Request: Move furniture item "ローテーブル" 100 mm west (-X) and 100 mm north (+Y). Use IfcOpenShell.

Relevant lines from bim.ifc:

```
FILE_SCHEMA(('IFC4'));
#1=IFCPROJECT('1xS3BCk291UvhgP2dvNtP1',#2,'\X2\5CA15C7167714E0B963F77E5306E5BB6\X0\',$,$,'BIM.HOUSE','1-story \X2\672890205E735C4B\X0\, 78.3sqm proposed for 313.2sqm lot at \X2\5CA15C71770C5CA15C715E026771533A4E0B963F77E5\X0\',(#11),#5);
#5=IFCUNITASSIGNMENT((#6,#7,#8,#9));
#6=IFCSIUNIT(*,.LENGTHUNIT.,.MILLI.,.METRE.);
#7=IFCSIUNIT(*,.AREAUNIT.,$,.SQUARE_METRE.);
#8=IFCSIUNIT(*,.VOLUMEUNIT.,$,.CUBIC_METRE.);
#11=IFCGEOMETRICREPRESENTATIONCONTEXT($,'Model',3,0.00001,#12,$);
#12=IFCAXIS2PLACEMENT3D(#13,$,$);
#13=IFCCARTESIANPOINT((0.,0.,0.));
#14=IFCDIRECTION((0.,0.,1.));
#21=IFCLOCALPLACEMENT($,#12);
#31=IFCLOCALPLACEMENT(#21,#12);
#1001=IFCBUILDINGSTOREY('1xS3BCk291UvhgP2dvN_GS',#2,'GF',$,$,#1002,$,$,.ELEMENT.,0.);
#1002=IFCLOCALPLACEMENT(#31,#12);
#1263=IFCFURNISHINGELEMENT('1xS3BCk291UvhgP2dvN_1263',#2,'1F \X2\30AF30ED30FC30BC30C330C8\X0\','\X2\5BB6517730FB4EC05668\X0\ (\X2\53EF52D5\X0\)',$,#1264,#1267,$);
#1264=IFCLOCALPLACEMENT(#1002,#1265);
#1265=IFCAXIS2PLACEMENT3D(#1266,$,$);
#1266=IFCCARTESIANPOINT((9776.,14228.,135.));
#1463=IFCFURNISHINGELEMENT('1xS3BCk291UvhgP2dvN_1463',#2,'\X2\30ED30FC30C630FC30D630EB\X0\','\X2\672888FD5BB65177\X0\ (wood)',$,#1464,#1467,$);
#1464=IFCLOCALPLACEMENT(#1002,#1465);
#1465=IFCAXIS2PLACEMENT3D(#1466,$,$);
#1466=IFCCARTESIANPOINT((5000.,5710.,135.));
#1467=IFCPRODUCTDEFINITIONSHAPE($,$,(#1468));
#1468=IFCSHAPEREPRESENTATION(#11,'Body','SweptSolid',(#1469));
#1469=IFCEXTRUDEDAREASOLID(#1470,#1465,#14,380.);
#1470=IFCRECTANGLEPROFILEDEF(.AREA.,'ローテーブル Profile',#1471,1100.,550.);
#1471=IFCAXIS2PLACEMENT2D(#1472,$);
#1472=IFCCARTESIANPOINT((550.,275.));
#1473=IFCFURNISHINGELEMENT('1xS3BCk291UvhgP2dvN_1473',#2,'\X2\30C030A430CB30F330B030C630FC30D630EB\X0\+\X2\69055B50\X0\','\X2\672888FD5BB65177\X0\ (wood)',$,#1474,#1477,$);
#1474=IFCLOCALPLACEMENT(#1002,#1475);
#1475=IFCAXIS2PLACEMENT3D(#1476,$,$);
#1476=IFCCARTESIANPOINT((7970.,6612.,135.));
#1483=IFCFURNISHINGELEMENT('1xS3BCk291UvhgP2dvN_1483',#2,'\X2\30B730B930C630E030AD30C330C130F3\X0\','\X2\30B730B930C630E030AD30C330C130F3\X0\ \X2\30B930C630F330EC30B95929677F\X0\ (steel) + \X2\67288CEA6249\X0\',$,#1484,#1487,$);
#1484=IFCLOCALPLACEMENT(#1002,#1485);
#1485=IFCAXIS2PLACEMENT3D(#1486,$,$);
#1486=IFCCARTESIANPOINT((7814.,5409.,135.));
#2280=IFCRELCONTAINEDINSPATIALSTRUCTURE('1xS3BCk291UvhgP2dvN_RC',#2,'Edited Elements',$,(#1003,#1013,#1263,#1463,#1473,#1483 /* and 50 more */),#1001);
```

```python
import ifcopenshell
import ifcopenshell.api.geometry
import ifcopenshell.util.placement
import ifcopenshell.util.unit

model = ifcopenshell.open("bim.ifc")
unit_scale = ifcopenshell.util.unit.calculate_unit_scale(model)

item = model.by_guid("1xS3BCk291UvhgP2dvN_1463")
matrix = ifcopenshell.util.placement.get_local_placement(item.ObjectPlacement)
matrix[0, 3] -= 0.1 / unit_scale
matrix[1, 3] += 0.1 / unit_scale
ifcopenshell.api.geometry.edit_object_placement(model, product=item, matrix=matrix, is_si=False)

print(ifcopenshell.util.placement.get_local_placement(item.ObjectPlacement).round(3) + 0.0)

model.write("bim_updated.ifc")
```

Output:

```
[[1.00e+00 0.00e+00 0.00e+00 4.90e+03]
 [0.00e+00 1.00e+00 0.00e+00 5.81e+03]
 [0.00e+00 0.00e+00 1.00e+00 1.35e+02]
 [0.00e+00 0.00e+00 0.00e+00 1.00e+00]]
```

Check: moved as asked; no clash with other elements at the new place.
